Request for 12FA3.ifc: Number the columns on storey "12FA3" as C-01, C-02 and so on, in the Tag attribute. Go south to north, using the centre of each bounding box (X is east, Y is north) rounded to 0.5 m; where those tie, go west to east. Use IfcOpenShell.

First a look at what the model holds.

```python
import ifcopenshell
import ifcopenshell.util.element
import ifcopenshell.util.placement

model = ifcopenshell.open("12FA3.ifc")
print(model.schema)
storey = next(s for s in model.by_type("IfcBuildingStorey") if s.Name == "12FA3")
columns = [e for e in ifcopenshell.util.element.get_decomposition(storey) if e.is_a("IfcColumn")]
for e in sorted(columns, key=lambda e: e.id()):
    origin = ifcopenshell.util.placement.get_local_placement(e.ObjectPlacement)[:3, 3]
    print(e.id(), e.Tag, e.Name, origin.round(2) + 0.0, sep=" | ")
```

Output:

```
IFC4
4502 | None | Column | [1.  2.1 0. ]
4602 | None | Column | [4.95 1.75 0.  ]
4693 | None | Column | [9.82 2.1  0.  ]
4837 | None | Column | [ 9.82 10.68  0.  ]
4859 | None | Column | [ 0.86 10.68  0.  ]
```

```python
import ifcopenshell
import ifcopenshell.geom
import ifcopenshell.util.element
import ifcopenshell.util.shape

model = ifcopenshell.open("12FA3.ifc")
settings = ifcopenshell.geom.settings()
settings.set("use-world-coords", True)


def centre(element):
    shape = ifcopenshell.geom.create_shape(settings, element)
    return ifcopenshell.util.shape.get_bbox_centroid(shape.geometry)


storey = next(s for s in model.by_type("IfcBuildingStorey") if s.Name == "12FA3")
columns = [e for e in ifcopenshell.util.element.get_decomposition(storey) if e.is_a("IfcColumn")]

# Insertion points can sit at a corner or the storey origin, so sort by the geometry (in metres).
centres = {e: centre(e) for e in columns}
columns.sort(key=lambda e: (round(centres[e][1] / 0.5), centres[e][0]))

for i, e in enumerate(columns, start=1):
    number = f"C-{i:02d}"
    e.Tag = number
    print(e.id(), number)

model.write("12FA3-out.ifc")
```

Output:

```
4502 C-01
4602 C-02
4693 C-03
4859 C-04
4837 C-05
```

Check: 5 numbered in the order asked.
